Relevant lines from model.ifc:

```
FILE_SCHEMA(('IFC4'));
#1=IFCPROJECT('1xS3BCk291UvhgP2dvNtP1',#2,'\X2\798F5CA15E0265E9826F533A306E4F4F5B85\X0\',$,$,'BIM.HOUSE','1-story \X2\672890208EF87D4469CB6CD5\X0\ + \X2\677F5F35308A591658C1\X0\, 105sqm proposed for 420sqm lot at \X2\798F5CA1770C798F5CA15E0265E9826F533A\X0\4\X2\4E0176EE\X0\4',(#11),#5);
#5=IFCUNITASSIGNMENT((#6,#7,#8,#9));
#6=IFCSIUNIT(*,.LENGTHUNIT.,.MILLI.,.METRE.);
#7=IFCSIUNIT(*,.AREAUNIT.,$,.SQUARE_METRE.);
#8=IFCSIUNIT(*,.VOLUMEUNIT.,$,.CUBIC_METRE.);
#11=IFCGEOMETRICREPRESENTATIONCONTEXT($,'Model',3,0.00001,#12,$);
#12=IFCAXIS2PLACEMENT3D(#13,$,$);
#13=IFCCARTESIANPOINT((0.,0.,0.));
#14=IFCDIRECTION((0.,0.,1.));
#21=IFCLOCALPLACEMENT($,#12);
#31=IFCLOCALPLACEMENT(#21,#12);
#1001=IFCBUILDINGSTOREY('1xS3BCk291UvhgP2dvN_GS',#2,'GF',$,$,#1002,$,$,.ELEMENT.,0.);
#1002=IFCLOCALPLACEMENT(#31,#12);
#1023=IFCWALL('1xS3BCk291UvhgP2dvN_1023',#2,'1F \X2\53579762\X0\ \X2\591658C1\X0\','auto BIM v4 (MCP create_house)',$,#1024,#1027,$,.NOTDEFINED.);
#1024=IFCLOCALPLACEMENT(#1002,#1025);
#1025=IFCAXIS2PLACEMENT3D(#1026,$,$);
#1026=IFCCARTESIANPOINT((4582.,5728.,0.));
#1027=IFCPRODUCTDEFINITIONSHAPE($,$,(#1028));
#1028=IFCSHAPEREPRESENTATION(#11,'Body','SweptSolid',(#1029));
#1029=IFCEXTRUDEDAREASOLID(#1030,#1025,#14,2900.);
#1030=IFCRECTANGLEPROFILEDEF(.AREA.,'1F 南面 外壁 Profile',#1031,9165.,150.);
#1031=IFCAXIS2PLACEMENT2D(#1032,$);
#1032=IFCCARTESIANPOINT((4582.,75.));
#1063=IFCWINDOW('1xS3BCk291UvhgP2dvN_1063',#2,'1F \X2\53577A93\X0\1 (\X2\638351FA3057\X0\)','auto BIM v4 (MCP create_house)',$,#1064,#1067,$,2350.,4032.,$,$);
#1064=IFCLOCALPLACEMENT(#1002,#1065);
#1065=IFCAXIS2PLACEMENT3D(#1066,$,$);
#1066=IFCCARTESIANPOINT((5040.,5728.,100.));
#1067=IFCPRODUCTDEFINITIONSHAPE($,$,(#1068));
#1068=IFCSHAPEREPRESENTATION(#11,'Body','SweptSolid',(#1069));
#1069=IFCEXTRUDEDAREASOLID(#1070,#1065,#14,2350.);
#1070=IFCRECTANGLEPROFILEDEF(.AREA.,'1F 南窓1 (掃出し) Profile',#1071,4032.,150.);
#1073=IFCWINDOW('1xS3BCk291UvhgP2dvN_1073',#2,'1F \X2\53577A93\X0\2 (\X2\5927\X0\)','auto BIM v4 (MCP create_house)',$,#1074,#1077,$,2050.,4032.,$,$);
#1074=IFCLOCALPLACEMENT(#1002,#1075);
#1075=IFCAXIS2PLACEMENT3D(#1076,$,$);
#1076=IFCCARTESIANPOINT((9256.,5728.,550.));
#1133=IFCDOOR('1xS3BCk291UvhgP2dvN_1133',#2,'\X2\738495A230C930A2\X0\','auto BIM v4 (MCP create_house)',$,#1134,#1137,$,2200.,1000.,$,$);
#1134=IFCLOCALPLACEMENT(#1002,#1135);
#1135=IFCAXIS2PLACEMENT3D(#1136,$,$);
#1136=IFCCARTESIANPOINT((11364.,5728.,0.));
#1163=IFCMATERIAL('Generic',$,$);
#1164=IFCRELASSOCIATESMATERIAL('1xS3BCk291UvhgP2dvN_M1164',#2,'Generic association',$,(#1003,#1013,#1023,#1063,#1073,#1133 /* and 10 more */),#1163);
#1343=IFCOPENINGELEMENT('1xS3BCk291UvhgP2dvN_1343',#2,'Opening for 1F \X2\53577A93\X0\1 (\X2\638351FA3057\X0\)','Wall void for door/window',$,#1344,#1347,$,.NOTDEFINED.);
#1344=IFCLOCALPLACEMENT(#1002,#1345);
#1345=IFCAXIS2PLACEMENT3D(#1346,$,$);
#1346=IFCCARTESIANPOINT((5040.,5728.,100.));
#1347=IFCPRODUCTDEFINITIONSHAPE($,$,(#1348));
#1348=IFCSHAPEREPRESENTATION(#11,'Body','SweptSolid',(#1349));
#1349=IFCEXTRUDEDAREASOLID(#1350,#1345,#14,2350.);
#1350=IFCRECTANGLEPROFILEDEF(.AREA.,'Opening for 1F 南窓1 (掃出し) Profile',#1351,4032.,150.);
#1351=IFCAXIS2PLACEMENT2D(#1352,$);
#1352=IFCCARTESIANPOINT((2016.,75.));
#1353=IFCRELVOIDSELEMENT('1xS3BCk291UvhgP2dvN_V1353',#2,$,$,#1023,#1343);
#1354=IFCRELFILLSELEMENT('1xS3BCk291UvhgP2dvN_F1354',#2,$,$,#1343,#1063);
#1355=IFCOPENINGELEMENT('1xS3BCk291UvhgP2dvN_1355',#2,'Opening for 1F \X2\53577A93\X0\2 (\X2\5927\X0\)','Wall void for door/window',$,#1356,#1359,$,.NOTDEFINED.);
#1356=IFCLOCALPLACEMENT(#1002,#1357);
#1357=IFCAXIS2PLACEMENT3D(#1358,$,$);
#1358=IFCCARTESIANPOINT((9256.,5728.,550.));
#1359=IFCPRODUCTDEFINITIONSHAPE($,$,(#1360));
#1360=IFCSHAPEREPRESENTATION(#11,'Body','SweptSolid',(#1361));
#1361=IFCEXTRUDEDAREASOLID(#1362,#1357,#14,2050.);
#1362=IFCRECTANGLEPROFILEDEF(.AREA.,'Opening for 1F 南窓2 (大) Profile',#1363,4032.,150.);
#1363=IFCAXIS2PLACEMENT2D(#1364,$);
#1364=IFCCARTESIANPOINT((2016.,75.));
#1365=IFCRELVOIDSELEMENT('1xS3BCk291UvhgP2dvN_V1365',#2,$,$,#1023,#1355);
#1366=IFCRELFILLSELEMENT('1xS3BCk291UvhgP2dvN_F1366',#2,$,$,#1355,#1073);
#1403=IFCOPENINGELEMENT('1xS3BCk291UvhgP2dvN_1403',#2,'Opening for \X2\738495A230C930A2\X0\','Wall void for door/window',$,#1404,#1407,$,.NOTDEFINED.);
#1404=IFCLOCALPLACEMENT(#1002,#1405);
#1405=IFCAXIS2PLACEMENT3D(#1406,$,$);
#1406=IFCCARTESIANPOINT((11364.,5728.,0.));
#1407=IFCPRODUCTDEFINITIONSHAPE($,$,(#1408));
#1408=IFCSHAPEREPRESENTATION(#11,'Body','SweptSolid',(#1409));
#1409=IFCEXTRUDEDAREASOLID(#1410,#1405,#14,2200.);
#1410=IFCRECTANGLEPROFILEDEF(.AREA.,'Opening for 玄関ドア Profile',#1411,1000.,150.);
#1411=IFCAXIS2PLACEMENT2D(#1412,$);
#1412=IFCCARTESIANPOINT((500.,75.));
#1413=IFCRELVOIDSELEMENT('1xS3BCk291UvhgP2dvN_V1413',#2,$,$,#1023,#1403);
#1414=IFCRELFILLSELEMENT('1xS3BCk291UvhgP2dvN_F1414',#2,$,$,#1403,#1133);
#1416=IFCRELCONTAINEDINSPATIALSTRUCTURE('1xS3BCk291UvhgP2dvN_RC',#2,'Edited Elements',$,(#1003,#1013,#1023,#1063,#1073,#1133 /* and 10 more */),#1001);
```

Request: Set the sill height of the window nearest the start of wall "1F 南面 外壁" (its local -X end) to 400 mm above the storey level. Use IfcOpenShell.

```python
import numpy as np
import ifcopenshell
import ifcopenshell.api.geometry
import ifcopenshell.geom
import ifcopenshell.util.element
import ifcopenshell.util.placement
import ifcopenshell.util.shape
import ifcopenshell.util.unit

model = ifcopenshell.open("model.ifc")
unit_scale = ifcopenshell.util.unit.calculate_unit_scale(model)

window = model.by_id(1063)
opening = window.FillsVoids[0].RelatingOpeningElement
storey = ifcopenshell.util.element.get_container(window, ifc_class="IfcBuildingStorey")
level = ifcopenshell.util.placement.get_local_placement(storey.ObjectPlacement)[2, 3]

# The opening's origin need not be at the sill, so measure its lowest point.
shape = ifcopenshell.geom.create_shape(ifcopenshell.geom.settings(), opening)
bottom = ifcopenshell.util.shape.get_shape_bottom_elevation(shape, shape.geometry) / unit_scale
dz = level + 0.4 / unit_scale - bottom

shift = np.array([0.0, 0.0, dz])
# The window is not placed relative to its opening, so move both.
for product in (opening, window):
    matrix = ifcopenshell.util.placement.get_local_placement(product.ObjectPlacement)
    matrix[:3, 3] += shift
    ifcopenshell.api.geometry.edit_object_placement(model, product=product, matrix=matrix, is_si=False)

print(f"moved by {dz * unit_scale:+.3f} m")

model.write("model-out.ifc")
```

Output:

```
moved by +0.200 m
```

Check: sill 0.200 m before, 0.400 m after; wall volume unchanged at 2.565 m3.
